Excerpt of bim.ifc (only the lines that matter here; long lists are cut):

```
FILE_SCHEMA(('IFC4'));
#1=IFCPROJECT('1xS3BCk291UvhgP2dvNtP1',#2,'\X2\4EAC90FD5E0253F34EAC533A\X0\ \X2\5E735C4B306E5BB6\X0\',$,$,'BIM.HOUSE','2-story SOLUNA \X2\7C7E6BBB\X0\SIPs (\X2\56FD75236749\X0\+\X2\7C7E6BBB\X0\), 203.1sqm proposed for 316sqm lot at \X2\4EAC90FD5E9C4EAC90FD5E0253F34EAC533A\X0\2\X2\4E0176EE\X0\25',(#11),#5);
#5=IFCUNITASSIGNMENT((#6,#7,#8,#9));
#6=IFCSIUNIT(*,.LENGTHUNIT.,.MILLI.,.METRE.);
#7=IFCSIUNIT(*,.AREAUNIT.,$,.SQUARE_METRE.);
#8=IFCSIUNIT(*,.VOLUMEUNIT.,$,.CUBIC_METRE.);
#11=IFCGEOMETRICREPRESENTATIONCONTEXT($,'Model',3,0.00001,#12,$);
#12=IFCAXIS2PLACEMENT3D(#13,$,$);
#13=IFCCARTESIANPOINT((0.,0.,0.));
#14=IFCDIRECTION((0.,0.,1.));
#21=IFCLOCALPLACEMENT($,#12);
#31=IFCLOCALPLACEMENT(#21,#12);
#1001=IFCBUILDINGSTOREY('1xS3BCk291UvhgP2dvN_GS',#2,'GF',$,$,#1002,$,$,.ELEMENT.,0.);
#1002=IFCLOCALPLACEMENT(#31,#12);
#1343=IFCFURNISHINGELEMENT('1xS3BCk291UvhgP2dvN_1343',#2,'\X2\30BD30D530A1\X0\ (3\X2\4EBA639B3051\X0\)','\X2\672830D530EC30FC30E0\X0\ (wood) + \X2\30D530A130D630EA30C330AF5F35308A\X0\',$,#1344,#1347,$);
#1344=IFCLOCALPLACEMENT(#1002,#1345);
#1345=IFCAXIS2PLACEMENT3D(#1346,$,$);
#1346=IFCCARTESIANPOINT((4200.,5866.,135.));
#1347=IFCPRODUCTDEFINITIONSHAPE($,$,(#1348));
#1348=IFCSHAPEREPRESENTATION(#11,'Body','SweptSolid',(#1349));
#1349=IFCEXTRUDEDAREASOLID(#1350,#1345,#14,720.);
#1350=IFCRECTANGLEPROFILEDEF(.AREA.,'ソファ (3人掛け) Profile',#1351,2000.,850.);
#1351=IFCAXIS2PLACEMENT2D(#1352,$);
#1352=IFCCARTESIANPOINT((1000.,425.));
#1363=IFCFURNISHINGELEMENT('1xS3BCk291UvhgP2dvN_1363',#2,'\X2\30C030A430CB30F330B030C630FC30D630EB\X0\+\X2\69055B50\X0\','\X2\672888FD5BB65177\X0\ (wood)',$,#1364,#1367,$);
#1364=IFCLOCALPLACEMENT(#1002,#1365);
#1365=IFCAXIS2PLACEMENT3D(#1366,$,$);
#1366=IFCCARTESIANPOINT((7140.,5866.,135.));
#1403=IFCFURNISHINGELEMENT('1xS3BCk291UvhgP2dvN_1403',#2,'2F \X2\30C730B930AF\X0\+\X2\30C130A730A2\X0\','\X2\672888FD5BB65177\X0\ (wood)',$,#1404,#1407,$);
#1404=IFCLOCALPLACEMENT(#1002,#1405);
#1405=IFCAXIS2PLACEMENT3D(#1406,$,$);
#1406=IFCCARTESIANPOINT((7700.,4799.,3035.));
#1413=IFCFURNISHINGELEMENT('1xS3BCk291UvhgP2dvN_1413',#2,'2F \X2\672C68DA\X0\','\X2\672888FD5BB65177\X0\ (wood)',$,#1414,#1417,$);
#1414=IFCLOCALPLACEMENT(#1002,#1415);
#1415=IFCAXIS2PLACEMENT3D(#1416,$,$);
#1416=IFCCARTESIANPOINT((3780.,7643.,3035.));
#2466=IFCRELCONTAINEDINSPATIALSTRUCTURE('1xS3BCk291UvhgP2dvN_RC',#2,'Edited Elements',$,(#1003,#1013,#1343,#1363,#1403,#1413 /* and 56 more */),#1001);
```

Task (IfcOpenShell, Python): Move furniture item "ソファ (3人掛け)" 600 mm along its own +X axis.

```python
import ifcopenshell
import ifcopenshell.api.geometry
import ifcopenshell.util.placement
import ifcopenshell.util.unit

model = ifcopenshell.open("bim.ifc")
unit_scale = ifcopenshell.util.unit.calculate_unit_scale(model)

item = model.by_guid("1xS3BCk291UvhgP2dvN_1343")
matrix = ifcopenshell.util.placement.get_local_placement(item.ObjectPlacement)
matrix[:3, 3] += matrix[:3, 0] * 0.6 / unit_scale
ifcopenshell.api.geometry.edit_object_placement(model, product=item, matrix=matrix, is_si=False)

print(ifcopenshell.util.placement.get_local_placement(item.ObjectPlacement).round(3) + 0.0)

model.write("bim-out.ifc")
```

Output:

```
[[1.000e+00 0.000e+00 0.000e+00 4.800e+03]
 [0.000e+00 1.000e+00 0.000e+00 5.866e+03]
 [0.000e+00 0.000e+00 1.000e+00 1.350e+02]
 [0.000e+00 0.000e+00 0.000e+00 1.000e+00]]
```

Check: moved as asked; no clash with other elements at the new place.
